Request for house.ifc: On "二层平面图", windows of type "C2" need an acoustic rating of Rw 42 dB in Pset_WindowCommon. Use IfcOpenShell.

First a look at what the model holds.

```python
import ifcopenshell
import ifcopenshell.util.element

model = ifcopenshell.open("house.ifc")
print(model.schema)
storey = next(s for s in model.by_type("IfcBuildingStorey") if s.Name == "二层平面图")
windows = [e for e in ifcopenshell.util.element.get_decomposition(storey) if e.is_a("IfcWindow")]
seen = {}
for e in windows:
    element_type = ifcopenshell.util.element.get_type(e)
    key = (element_type.Name if element_type != e and element_type else None, ifcopenshell.util.element.get_pset(e, "Pset_WindowCommon", "AcousticRating"))
    seen[key] = seen.get(key, 0) + 1
for (name, value), count in sorted(seen.items(), key=str):
    print(count, "x", name, "|", value)
```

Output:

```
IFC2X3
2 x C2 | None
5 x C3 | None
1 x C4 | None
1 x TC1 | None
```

```python
import ifcopenshell
import ifcopenshell.api.pset
import ifcopenshell.util.element

model = ifcopenshell.open("house.ifc")

storey = next(s for s in model.by_type("IfcBuildingStorey") if s.Name == "二层平面图")
windows = [e for e in ifcopenshell.util.element.get_decomposition(storey) if e.is_a("IfcWindow")]

count = 0
for e in windows:
    element_type = ifcopenshell.util.element.get_type(e)
    if element_type in (None, e) or element_type.Name != "C2":
        continue
    # add_pset returns the element's existing set when there is one.
    pset = ifcopenshell.api.pset.add_pset(model, product=e, name="Pset_WindowCommon")
    ifcopenshell.api.pset.edit_pset(model, pset=pset, properties={"AcousticRating": "Rw 42 dB"})
    count += 1

print(count, "windows updated")

model.write("house_rev.ifc")
```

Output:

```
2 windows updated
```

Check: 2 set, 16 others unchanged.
